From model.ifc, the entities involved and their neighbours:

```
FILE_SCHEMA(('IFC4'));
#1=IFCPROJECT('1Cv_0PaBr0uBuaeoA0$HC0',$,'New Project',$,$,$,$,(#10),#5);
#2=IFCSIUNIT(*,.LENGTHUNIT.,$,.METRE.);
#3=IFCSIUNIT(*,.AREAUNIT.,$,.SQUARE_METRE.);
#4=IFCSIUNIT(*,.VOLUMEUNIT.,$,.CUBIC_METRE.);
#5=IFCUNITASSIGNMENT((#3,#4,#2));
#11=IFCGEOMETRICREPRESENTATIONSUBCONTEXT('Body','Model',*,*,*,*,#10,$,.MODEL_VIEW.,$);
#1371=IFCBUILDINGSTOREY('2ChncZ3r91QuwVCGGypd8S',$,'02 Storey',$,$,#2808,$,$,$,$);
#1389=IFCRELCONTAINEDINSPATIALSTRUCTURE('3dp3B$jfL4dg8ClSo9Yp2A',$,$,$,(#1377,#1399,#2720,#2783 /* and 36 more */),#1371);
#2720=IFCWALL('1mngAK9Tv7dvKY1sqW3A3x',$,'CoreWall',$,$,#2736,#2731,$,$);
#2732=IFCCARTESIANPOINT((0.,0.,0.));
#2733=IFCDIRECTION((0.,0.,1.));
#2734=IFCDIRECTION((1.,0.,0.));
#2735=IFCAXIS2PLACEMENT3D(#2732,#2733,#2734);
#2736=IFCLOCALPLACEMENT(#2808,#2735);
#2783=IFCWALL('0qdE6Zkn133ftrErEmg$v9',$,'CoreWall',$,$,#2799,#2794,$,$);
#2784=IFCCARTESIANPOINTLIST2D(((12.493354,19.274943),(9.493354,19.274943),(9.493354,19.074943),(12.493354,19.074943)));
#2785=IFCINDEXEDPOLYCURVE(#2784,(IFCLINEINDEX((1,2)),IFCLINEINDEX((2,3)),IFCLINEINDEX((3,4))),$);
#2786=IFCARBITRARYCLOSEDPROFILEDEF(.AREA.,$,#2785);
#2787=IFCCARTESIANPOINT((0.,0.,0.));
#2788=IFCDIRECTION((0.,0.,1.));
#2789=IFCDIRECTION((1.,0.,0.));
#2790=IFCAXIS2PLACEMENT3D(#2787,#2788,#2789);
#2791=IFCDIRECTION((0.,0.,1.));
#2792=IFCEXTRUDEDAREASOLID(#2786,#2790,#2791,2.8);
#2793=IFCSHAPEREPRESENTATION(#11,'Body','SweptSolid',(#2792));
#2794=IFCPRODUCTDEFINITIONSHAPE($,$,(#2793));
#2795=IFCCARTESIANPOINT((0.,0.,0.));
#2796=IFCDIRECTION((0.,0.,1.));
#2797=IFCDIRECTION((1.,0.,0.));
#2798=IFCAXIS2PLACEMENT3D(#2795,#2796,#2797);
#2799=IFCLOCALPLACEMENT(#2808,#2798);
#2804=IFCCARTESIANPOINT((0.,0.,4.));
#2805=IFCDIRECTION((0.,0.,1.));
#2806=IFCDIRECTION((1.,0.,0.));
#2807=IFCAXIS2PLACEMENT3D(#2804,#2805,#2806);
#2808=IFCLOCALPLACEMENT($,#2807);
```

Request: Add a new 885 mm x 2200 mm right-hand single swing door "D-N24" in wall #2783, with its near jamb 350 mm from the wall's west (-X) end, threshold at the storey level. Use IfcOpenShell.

```python
import numpy as np
import ifcopenshell
import ifcopenshell.api.feature
import ifcopenshell.api.geometry
import ifcopenshell.api.root
import ifcopenshell.api.spatial
import ifcopenshell.geom
import ifcopenshell.util.element
import ifcopenshell.util.placement
import ifcopenshell.util.representation
import ifcopenshell.util.shape
import ifcopenshell.util.unit

model = ifcopenshell.open("model.ifc")
unit_scale = ifcopenshell.util.unit.calculate_unit_scale(model)
settings = ifcopenshell.geom.settings()


def volume(element):
    """Net volume in cubic metres, openings subtracted."""
    shape = ifcopenshell.geom.create_shape(settings, element)
    return ifcopenshell.util.shape.get_volume(shape.geometry)


wall = model.by_guid("0qdE6Zkn133ftrErEmg$v9")
storey = ifcopenshell.util.element.get_container(wall, ifc_class="IfcBuildingStorey")
context = ifcopenshell.util.representation.get_context(model, "Model", "Body", "MODEL_VIEW")
before = volume(wall)

width, height, from_end, sill = 0.885, 2.2, 0.35, 0.0  # metres

# The wall runs along its own X axis, and the end named is its -X end.
wall_shape = ifcopenshell.geom.create_shape(settings, wall)
x, y, z = ifcopenshell.util.shape.get_vertices(wall_shape.geometry).T
start = x.min() + from_end
face, thickness = float(y.min()), float(y.max() - y.min())
wall_matrix = ifcopenshell.util.placement.get_local_placement(wall.ObjectPlacement)
level = ifcopenshell.util.placement.get_local_placement(storey.ObjectPlacement)[2, 3]


def in_wall(x, y):
    """Placement at x, y metres in the wall's axes, at sill height."""
    matrix = wall_matrix.copy()
    matrix[:, 3] = wall_matrix @ np.array([x / unit_scale, y / unit_scale, 0.0, 1.0])
    matrix[2, 3] = level + sill / unit_scale
    return matrix


# Opening: a box that overshoots both wall faces by 50 mm.
opening = ifcopenshell.api.root.create_entity(model, ifc_class="IfcOpeningElement", predefined_type="OPENING")
box = ifcopenshell.api.geometry.add_wall_representation(
    model, context=context, length=width, height=height, thickness=thickness + 0.1
)
ifcopenshell.api.geometry.assign_representation(model, product=opening, representation=box)
ifcopenshell.api.geometry.edit_object_placement(model, product=opening, matrix=in_wall(start, face - 0.05), is_si=False)
ifcopenshell.api.feature.add_feature(model, feature=opening, element=wall)

door = ifcopenshell.api.root.create_entity(model, ifc_class="IfcDoor", name="D-N24", predefined_type="DOOR")
door.OverallWidth, door.OverallHeight = width / unit_scale, height / unit_scale
door.OperationType = "SINGLE_SWING_RIGHT"
body = ifcopenshell.api.geometry.add_door_representation(
    model,
    context=context,
    overall_width=door.OverallWidth,
    overall_height=door.OverallHeight,
    operation_type="SINGLE_SWING_RIGHT",
    lining_properties={"LiningDepth": thickness / unit_scale, "ThresholdDepth": thickness / unit_scale},
)
ifcopenshell.api.geometry.assign_representation(model, product=door, representation=body)
ifcopenshell.api.spatial.assign_container(model, products=[door], relating_structure=storey)
ifcopenshell.api.feature.add_filling(model, opening=opening, element=door)

# The lining spans the wall, so the door starts at the wall face.
ifcopenshell.api.geometry.edit_object_placement(model, product=door, matrix=in_wall(start, face), is_si=False)

after = volume(wall)

print(f"wall volume {before:.3f} -> {after:.3f} m3")

model.write("model_rev.ifc")
```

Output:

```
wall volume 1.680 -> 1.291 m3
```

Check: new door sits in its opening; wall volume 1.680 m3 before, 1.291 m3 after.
